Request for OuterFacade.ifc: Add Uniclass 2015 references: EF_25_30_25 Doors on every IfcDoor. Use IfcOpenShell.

First a look at what the model holds.

```python
import ifcopenshell

model = ifcopenshell.open("OuterFacade.ifc")
print(model.schema)
print("classifications:", [c.Name for c in model.by_type("IfcClassification")])
for ifc_class in ("IfcDoor", "IfcRoof", "IfcStair", "IfcWall", "IfcWindow"):
    print(ifc_class, len(model.by_type(ifc_class)))
```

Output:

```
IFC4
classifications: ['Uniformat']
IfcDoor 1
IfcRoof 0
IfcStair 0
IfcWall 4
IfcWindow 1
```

```python
import ifcopenshell
import ifcopenshell.api.classification

model = ifcopenshell.open("OuterFacade.ifc")

system = ifcopenshell.api.classification.add_classification(model, classification="Uniclass 2015")

codes = {
    "IfcDoor": ("EF_25_30_25", "Doors"),
}
for ifc_class, (code, name) in codes.items():
    products = model.by_type(ifc_class)
    ifcopenshell.api.classification.add_reference(
        model, products=products, classification=system, identification=code, name=name
    )
    print(code, len(products))

model.write("OuterFacade_v2.ifc")
```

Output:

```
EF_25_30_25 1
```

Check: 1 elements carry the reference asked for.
